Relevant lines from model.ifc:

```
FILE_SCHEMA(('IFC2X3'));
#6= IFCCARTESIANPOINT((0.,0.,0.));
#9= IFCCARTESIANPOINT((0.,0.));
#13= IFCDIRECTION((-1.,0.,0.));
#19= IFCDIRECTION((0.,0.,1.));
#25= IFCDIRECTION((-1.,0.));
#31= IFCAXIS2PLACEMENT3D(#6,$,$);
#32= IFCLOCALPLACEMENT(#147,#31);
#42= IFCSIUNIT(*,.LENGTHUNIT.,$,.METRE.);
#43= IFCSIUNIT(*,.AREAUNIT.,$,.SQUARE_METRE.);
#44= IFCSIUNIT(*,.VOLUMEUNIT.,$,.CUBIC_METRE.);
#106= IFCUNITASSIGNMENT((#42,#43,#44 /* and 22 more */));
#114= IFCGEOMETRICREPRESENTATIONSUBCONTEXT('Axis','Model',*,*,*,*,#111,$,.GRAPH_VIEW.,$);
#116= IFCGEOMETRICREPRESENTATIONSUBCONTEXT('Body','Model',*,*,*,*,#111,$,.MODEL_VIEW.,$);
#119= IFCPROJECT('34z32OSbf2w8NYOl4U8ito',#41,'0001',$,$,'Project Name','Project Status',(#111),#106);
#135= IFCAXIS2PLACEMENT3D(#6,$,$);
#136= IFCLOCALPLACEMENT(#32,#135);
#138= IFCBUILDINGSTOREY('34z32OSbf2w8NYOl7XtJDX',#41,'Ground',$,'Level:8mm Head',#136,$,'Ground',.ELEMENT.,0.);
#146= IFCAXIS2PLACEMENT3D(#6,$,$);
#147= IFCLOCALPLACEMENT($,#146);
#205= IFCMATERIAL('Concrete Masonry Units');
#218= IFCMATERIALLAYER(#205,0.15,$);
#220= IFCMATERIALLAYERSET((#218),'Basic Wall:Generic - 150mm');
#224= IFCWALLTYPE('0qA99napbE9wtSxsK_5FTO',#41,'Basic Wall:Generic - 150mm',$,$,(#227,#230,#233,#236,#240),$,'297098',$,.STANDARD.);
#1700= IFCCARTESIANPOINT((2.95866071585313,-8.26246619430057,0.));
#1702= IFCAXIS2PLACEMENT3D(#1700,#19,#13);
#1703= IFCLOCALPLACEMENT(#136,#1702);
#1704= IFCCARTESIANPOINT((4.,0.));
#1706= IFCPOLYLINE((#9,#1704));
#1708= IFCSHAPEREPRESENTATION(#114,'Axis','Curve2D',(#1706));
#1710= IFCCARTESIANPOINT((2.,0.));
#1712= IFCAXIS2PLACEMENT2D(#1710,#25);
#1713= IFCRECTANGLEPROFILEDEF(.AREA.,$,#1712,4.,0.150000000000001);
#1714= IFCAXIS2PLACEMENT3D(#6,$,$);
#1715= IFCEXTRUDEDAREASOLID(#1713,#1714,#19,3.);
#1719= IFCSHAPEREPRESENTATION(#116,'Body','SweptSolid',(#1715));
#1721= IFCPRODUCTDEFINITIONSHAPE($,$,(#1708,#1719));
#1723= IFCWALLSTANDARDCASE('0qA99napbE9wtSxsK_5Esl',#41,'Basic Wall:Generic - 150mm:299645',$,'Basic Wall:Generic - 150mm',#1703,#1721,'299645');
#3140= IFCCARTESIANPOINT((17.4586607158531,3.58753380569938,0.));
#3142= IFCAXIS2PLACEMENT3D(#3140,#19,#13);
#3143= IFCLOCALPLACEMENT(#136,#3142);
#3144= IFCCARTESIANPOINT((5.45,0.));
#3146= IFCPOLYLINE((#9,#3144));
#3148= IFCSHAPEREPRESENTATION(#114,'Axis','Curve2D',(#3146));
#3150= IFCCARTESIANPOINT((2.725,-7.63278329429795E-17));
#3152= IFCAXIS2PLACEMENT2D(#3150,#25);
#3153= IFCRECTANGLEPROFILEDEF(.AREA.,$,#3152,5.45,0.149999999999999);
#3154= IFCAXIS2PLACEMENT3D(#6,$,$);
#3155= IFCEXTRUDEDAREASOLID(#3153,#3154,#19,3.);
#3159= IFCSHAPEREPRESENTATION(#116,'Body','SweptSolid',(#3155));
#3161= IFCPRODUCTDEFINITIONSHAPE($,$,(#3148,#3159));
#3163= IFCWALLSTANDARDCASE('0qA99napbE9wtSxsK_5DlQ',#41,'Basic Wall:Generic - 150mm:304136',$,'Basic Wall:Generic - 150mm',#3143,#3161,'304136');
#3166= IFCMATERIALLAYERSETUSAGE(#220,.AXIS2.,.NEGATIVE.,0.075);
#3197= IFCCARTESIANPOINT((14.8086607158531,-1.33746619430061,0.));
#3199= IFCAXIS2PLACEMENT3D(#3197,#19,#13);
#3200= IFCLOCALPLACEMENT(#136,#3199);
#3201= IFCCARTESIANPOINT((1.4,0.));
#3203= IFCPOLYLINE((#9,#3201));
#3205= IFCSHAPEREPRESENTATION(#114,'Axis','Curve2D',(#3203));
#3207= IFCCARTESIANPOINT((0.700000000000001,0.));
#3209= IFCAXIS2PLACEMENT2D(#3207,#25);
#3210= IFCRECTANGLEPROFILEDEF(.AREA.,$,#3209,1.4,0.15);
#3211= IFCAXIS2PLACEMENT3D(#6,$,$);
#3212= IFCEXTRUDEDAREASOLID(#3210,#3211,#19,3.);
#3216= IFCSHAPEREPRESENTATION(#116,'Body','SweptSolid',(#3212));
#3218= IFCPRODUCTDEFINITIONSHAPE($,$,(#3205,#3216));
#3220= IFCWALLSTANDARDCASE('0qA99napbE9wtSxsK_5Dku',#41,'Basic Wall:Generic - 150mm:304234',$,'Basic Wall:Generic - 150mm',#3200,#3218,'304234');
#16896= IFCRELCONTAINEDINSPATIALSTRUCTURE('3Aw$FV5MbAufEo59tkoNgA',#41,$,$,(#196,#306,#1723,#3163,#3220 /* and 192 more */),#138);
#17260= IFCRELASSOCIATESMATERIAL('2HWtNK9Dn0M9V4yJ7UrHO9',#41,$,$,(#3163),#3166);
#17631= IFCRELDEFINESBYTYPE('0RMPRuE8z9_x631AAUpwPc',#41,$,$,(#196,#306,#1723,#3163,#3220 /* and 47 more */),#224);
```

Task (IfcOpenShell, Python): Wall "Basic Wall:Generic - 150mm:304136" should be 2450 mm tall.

```python
import ifcopenshell
import ifcopenshell.geom
import ifcopenshell.util.representation
import ifcopenshell.util.shape
import ifcopenshell.util.unit

model = ifcopenshell.open("model.ifc")
unit_scale = ifcopenshell.util.unit.calculate_unit_scale(model)
settings = ifcopenshell.geom.settings()


def volume(element):
    """Net volume in cubic metres, openings subtracted."""
    shape = ifcopenshell.geom.create_shape(settings, element)
    return ifcopenshell.util.shape.get_volume(shape.geometry)


wall = model.by_guid("0qA99napbE9wtSxsK_5DlQ")
before = volume(wall)

body = ifcopenshell.util.representation.get_representation(wall, "Model", "Body")
solid = body.Items[0]
old_height = solid.Depth
solid.Depth = 2.45 / unit_scale
after = volume(wall)

print(f"height {old_height:g} -> {solid.Depth:g}, volume {before:.3f} -> {after:.3f} m3")

model.write("model_updated.ifc")
```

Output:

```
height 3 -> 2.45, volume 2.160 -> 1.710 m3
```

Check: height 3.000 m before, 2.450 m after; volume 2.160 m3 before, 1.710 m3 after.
